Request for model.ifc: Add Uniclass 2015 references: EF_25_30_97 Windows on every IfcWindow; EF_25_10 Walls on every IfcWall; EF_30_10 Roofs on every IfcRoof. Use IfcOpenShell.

First a look at what the model holds.

```python
import ifcopenshell

model = ifcopenshell.open("model.ifc")
print(model.schema)
print("classifications:", [c.Name for c in model.by_type("IfcClassification")])
for ifc_class in ("IfcDoor", "IfcRoof", "IfcStair", "IfcWall", "IfcWindow"):
    print(ifc_class, len(model.by_type(ifc_class)))
```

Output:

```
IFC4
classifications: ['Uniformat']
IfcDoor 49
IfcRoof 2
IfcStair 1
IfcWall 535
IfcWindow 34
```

```python
import ifcopenshell
import ifcopenshell.api.classification

model = ifcopenshell.open("model.ifc")

system = ifcopenshell.api.classification.add_classification(model, classification="Uniclass 2015")

codes = {
    "IfcWindow": ("EF_25_30_97", "Windows"),
    "IfcWall": ("EF_25_10", "Walls"),
    "IfcRoof": ("EF_30_10", "Roofs"),
}
for ifc_class, (code, name) in codes.items():
    products = model.by_type(ifc_class)
    ifcopenshell.api.classification.add_reference(
        model, products=products, classification=system, identification=code, name=name
    )
    print(code, len(products))

model.write("model_rev.ifc")
```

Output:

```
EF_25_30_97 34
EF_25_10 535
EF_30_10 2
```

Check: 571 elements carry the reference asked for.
